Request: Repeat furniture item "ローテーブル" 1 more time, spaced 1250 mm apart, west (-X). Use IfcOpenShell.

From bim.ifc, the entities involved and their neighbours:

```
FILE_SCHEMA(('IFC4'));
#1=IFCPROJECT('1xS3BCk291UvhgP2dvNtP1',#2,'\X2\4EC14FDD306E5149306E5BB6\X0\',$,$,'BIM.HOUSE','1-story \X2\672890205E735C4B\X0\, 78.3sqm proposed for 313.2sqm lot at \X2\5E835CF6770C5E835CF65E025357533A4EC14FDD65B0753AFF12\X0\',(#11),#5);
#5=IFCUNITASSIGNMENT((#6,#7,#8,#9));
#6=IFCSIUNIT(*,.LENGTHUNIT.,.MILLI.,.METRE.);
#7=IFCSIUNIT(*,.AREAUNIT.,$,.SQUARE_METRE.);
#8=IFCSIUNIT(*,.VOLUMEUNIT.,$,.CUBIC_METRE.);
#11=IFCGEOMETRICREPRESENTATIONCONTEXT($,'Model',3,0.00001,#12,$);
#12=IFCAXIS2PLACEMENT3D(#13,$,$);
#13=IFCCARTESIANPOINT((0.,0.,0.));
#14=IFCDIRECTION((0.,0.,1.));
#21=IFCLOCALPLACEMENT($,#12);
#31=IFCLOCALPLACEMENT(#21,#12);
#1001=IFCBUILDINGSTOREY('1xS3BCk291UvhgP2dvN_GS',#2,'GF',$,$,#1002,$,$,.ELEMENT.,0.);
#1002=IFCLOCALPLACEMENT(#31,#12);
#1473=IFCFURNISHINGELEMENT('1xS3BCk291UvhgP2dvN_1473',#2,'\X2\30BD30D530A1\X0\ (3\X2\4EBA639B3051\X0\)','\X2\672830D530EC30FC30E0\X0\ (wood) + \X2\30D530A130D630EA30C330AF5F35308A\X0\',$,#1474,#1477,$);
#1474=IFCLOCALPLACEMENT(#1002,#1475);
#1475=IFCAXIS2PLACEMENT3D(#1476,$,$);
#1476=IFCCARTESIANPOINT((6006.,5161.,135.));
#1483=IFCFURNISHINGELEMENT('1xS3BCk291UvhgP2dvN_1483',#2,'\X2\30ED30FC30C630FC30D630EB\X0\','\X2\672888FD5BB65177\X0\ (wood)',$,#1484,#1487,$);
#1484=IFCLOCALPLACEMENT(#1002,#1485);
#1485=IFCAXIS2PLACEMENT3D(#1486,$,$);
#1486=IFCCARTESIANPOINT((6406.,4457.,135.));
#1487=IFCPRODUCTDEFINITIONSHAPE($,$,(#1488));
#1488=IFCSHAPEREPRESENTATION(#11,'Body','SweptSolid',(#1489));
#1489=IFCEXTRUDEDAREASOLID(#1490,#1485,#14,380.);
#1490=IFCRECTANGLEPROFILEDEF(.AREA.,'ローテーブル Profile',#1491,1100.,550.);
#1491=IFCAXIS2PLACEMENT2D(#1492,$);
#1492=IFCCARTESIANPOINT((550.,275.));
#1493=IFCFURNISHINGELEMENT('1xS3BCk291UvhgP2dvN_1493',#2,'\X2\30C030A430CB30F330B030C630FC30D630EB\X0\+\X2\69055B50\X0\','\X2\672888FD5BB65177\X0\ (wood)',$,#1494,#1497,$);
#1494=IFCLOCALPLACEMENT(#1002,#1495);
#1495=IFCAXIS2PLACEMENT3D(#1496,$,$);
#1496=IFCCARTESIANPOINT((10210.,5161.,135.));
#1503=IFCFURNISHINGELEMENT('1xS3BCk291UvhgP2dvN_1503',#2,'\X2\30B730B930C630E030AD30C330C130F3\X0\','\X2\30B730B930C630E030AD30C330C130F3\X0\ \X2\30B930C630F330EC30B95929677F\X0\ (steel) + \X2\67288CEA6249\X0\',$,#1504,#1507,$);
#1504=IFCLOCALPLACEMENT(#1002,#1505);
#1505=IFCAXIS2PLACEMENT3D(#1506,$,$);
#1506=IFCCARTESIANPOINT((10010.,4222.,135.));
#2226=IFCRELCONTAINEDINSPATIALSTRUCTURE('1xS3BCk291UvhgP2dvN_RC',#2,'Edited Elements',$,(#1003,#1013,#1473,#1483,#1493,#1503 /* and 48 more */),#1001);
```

```python
import numpy as np
import ifcopenshell
import ifcopenshell.api.geometry
import ifcopenshell.api.root
import ifcopenshell.util.element
import ifcopenshell.util.placement
import ifcopenshell.util.unit

model = ifcopenshell.open("bim.ifc")
unit_scale = ifcopenshell.util.unit.calculate_unit_scale(model)


def reuse_history(source, copy):
    """copy_class also copies each property set's owner history, people and application; keep the originals."""
    for rel in copy.IsDefinedBy:
        if rel.is_a("IfcRelDefinesByProperties") and (history := rel.RelatingPropertyDefinition.OwnerHistory):
            rel.RelatingPropertyDefinition.OwnerHistory = source.OwnerHistory
            ifcopenshell.util.element.remove_deep2(model, history)


source = model.by_guid("1xS3BCk291UvhgP2dvN_1483")
base = ifcopenshell.util.placement.get_local_placement(source.ObjectPlacement)
step = np.array([-1.0, 0.0, 0.0]) * 1.25 / unit_scale

for i in range(1, 2):
    copy = ifcopenshell.api.root.copy_class(model, product=source)
    copy.Representation = ifcopenshell.util.element.copy_deep(
        model, source.Representation, exclude=["IfcGeometricRepresentationContext", "IfcRepresentationMap"]
    )
    reuse_history(source, copy)
    matrix = base.copy()
    matrix[:3, 3] += i * step
    print("added at", matrix[:3, 3].round(3) + 0.0)
    ifcopenshell.api.geometry.edit_object_placement(model, product=copy, matrix=matrix, is_si=False)

model.write("bim-out.ifc")
```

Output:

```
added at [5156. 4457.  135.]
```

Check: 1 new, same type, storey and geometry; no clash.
